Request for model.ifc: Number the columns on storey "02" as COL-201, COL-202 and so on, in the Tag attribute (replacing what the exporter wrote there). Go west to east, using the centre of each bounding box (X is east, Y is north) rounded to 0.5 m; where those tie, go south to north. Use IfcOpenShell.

First a look at what the model holds.

```python
import ifcopenshell
import ifcopenshell.util.element
import ifcopenshell.util.placement

model = ifcopenshell.open("model.ifc")
print(model.schema)
storey = next(s for s in model.by_type("IfcBuildingStorey") if s.Name == "02")
columns = [e for e in ifcopenshell.util.element.get_decomposition(storey) if e.is_a("IfcColumn")]
for e in sorted(columns, key=lambda e: e.id()):
    origin = ifcopenshell.util.placement.get_local_placement(e.ObjectPlacement)[:3, 3]
    print(e.id(), e.Tag, e.Name, origin.round(2) + 0.0, sep=" | ")
```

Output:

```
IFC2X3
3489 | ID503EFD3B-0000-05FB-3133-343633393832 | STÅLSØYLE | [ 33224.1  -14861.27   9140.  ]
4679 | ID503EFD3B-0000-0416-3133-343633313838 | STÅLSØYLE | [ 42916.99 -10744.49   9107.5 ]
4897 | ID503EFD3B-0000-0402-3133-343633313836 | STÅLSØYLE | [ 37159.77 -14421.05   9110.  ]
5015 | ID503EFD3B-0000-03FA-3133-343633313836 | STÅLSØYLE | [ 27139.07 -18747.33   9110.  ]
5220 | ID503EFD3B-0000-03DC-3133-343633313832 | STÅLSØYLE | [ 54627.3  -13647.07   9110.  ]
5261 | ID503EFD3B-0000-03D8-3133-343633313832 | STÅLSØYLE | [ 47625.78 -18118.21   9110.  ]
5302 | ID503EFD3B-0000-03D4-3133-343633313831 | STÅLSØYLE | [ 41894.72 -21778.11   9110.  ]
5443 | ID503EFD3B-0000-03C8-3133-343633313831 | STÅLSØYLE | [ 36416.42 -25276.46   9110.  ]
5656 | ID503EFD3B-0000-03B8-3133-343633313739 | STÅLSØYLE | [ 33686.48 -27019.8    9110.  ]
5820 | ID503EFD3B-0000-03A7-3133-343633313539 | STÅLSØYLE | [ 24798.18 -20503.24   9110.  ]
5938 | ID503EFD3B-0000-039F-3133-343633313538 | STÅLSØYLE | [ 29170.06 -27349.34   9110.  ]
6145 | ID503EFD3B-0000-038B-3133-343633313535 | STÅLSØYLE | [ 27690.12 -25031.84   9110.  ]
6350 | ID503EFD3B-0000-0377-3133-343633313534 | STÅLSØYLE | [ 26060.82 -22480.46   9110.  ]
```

```python
import ifcopenshell
import ifcopenshell.geom
import ifcopenshell.util.element
import ifcopenshell.util.shape

model = ifcopenshell.open("model.ifc")
settings = ifcopenshell.geom.settings()
settings.set("use-world-coords", True)


def centre(element):
    shape = ifcopenshell.geom.create_shape(settings, element)
    return ifcopenshell.util.shape.get_bbox_centroid(shape.geometry)


storey = next(s for s in model.by_type("IfcBuildingStorey") if s.Name == "02")
columns = [e for e in ifcopenshell.util.element.get_decomposition(storey) if e.is_a("IfcColumn")]

# Insertion points can sit at a corner or the storey origin, so sort by the geometry (in metres).
centres = {e: centre(e) for e in columns}
columns.sort(key=lambda e: (round(centres[e][0] / 0.5), centres[e][1]))

for i, e in enumerate(columns, start=1):
    number = f"COL-2{i:02d}"
    e.Tag = number
    print(e.id(), number)

model.write("model_edited.ifc")
```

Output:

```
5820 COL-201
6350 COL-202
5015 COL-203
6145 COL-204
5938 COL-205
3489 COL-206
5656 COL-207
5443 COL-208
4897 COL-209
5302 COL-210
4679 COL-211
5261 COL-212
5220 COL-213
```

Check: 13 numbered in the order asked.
